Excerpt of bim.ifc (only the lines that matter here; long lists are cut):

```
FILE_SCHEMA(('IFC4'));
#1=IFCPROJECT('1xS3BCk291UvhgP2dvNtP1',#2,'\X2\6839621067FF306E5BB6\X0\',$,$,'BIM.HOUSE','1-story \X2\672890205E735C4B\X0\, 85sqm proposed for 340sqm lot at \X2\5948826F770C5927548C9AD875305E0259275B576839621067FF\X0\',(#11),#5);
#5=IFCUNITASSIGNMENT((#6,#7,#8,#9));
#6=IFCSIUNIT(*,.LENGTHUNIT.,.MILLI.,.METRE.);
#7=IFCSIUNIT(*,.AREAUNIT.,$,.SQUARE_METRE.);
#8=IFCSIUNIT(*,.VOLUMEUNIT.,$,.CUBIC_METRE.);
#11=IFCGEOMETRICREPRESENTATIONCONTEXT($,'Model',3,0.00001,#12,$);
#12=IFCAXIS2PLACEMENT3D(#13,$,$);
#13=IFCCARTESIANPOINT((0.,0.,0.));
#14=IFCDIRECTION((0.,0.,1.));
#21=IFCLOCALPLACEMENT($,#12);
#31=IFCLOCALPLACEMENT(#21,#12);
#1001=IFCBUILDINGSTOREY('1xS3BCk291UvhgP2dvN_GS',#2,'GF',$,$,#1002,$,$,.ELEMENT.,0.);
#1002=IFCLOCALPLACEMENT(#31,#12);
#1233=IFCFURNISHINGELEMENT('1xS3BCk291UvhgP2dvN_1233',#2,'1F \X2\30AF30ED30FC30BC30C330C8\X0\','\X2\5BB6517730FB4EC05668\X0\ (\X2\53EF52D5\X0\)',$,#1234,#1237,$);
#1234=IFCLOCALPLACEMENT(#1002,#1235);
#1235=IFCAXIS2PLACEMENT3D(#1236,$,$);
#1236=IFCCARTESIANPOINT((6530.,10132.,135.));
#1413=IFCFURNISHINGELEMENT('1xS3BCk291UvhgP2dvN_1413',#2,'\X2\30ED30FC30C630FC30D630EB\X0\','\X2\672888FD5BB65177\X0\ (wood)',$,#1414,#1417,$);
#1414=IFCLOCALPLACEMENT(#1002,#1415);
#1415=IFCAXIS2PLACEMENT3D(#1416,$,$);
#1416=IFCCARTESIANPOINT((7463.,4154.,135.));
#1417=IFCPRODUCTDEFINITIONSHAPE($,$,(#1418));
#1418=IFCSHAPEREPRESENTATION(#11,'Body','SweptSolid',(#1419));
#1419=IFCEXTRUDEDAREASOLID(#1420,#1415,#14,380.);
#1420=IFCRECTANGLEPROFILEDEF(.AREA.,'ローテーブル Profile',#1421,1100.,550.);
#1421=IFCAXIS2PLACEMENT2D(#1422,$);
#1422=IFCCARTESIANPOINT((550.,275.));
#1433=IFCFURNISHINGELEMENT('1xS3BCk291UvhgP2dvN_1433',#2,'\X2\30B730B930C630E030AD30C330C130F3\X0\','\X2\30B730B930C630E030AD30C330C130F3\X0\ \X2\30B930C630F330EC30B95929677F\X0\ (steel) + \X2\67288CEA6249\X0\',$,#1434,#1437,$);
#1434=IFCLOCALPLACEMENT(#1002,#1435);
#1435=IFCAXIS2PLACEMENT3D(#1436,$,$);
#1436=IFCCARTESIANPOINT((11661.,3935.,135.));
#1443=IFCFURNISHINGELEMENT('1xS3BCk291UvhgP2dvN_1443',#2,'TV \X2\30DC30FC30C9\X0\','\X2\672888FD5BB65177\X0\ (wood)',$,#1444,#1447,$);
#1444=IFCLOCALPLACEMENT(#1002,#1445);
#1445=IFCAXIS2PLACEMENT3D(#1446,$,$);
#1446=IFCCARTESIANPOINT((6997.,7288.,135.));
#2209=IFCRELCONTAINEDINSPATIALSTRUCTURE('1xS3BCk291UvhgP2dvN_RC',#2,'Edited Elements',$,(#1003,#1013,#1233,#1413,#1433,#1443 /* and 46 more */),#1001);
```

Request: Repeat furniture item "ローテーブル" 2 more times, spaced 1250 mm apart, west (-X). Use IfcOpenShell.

```python
import numpy as np
import ifcopenshell
import ifcopenshell.api.geometry
import ifcopenshell.api.root
import ifcopenshell.util.element
import ifcopenshell.util.placement
import ifcopenshell.util.unit

model = ifcopenshell.open("bim.ifc")
unit_scale = ifcopenshell.util.unit.calculate_unit_scale(model)


def reuse_history(source, copy):
    """copy_class also copies each property set's owner history, people and application; keep the originals."""
    for rel in copy.IsDefinedBy:
        if rel.is_a("IfcRelDefinesByProperties") and (history := rel.RelatingPropertyDefinition.OwnerHistory):
            rel.RelatingPropertyDefinition.OwnerHistory = source.OwnerHistory
            ifcopenshell.util.element.remove_deep2(model, history)


source = model.by_guid("1xS3BCk291UvhgP2dvN_1413")
base = ifcopenshell.util.placement.get_local_placement(source.ObjectPlacement)
step = np.array([-1.0, 0.0, 0.0]) * 1.25 / unit_scale

for i in range(1, 3):
    copy = ifcopenshell.api.root.copy_class(model, product=source)
    copy.Representation = ifcopenshell.util.element.copy_deep(
        model, source.Representation, exclude=["IfcGeometricRepresentationContext", "IfcRepresentationMap"]
    )
    reuse_history(source, copy)
    matrix = base.copy()
    matrix[:3, 3] += i * step
    print("added at", matrix[:3, 3].round(3) + 0.0)
    ifcopenshell.api.geometry.edit_object_placement(model, product=copy, matrix=matrix, is_si=False)

model.write("bim_rev.ifc")
```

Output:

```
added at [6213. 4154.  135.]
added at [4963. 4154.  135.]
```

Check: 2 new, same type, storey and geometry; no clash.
